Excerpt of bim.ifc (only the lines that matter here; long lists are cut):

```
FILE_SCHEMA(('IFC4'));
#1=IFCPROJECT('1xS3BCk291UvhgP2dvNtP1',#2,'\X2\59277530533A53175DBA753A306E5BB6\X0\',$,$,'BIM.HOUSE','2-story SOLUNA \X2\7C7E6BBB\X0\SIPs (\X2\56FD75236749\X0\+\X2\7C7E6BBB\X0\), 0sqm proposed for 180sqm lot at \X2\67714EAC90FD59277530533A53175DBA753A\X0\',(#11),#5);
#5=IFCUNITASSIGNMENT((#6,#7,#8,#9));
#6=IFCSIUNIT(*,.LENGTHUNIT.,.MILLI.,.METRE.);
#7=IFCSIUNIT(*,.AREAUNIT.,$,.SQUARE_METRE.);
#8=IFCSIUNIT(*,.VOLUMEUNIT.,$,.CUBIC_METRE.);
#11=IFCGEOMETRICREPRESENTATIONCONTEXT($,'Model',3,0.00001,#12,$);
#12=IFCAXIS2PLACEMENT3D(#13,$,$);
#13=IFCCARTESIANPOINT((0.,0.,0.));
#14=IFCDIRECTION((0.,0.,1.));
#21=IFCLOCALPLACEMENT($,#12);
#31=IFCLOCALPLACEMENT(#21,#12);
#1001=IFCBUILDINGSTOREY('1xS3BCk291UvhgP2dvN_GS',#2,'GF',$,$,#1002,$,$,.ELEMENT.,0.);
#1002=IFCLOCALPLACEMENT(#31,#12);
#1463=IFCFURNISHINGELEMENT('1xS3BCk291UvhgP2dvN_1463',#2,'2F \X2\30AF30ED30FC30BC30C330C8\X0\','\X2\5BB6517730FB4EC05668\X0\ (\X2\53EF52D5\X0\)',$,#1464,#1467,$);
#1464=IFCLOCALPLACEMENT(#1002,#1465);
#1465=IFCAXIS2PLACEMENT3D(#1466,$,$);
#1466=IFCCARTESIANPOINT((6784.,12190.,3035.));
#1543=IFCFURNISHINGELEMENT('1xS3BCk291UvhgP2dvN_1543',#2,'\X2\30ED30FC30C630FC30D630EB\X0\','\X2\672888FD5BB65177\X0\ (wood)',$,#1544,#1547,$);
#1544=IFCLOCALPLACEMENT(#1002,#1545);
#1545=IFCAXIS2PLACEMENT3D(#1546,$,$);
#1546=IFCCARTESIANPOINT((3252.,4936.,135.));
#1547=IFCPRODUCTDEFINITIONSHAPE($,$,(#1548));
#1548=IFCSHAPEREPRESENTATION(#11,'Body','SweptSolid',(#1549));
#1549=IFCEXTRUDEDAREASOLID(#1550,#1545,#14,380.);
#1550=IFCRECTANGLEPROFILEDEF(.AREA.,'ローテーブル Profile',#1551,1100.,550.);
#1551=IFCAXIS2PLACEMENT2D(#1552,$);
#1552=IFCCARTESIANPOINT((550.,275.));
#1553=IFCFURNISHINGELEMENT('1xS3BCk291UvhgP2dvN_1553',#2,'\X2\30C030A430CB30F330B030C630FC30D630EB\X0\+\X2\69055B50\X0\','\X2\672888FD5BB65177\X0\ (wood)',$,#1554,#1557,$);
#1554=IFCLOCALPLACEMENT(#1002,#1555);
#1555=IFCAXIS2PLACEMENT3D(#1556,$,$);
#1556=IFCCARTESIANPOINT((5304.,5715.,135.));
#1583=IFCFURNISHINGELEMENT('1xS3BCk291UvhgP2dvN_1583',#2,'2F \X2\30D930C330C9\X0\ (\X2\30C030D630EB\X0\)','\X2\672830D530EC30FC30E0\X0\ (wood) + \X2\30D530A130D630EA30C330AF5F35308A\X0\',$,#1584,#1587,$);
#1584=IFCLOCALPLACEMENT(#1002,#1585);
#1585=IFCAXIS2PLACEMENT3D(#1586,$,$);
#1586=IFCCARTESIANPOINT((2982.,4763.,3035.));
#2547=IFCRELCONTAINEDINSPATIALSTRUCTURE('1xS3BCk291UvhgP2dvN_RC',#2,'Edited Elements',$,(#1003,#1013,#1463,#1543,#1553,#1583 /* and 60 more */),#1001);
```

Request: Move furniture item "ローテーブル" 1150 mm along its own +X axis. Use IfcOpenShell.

```python
import ifcopenshell
import ifcopenshell.api.geometry
import ifcopenshell.util.placement
import ifcopenshell.util.unit

model = ifcopenshell.open("bim.ifc")
unit_scale = ifcopenshell.util.unit.calculate_unit_scale(model)

item = model.by_id(1543)
matrix = ifcopenshell.util.placement.get_local_placement(item.ObjectPlacement)
matrix[:3, 3] += matrix[:3, 0] * 1.15 / unit_scale
ifcopenshell.api.geometry.edit_object_placement(model, product=item, matrix=matrix, is_si=False)

print(ifcopenshell.util.placement.get_local_placement(item.ObjectPlacement).round(3) + 0.0)

model.write("bim_rev.ifc")
```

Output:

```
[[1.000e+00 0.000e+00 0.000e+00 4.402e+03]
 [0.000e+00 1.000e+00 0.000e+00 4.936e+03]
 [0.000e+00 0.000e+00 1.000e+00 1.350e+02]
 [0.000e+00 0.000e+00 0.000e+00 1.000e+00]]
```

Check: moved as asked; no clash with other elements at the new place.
